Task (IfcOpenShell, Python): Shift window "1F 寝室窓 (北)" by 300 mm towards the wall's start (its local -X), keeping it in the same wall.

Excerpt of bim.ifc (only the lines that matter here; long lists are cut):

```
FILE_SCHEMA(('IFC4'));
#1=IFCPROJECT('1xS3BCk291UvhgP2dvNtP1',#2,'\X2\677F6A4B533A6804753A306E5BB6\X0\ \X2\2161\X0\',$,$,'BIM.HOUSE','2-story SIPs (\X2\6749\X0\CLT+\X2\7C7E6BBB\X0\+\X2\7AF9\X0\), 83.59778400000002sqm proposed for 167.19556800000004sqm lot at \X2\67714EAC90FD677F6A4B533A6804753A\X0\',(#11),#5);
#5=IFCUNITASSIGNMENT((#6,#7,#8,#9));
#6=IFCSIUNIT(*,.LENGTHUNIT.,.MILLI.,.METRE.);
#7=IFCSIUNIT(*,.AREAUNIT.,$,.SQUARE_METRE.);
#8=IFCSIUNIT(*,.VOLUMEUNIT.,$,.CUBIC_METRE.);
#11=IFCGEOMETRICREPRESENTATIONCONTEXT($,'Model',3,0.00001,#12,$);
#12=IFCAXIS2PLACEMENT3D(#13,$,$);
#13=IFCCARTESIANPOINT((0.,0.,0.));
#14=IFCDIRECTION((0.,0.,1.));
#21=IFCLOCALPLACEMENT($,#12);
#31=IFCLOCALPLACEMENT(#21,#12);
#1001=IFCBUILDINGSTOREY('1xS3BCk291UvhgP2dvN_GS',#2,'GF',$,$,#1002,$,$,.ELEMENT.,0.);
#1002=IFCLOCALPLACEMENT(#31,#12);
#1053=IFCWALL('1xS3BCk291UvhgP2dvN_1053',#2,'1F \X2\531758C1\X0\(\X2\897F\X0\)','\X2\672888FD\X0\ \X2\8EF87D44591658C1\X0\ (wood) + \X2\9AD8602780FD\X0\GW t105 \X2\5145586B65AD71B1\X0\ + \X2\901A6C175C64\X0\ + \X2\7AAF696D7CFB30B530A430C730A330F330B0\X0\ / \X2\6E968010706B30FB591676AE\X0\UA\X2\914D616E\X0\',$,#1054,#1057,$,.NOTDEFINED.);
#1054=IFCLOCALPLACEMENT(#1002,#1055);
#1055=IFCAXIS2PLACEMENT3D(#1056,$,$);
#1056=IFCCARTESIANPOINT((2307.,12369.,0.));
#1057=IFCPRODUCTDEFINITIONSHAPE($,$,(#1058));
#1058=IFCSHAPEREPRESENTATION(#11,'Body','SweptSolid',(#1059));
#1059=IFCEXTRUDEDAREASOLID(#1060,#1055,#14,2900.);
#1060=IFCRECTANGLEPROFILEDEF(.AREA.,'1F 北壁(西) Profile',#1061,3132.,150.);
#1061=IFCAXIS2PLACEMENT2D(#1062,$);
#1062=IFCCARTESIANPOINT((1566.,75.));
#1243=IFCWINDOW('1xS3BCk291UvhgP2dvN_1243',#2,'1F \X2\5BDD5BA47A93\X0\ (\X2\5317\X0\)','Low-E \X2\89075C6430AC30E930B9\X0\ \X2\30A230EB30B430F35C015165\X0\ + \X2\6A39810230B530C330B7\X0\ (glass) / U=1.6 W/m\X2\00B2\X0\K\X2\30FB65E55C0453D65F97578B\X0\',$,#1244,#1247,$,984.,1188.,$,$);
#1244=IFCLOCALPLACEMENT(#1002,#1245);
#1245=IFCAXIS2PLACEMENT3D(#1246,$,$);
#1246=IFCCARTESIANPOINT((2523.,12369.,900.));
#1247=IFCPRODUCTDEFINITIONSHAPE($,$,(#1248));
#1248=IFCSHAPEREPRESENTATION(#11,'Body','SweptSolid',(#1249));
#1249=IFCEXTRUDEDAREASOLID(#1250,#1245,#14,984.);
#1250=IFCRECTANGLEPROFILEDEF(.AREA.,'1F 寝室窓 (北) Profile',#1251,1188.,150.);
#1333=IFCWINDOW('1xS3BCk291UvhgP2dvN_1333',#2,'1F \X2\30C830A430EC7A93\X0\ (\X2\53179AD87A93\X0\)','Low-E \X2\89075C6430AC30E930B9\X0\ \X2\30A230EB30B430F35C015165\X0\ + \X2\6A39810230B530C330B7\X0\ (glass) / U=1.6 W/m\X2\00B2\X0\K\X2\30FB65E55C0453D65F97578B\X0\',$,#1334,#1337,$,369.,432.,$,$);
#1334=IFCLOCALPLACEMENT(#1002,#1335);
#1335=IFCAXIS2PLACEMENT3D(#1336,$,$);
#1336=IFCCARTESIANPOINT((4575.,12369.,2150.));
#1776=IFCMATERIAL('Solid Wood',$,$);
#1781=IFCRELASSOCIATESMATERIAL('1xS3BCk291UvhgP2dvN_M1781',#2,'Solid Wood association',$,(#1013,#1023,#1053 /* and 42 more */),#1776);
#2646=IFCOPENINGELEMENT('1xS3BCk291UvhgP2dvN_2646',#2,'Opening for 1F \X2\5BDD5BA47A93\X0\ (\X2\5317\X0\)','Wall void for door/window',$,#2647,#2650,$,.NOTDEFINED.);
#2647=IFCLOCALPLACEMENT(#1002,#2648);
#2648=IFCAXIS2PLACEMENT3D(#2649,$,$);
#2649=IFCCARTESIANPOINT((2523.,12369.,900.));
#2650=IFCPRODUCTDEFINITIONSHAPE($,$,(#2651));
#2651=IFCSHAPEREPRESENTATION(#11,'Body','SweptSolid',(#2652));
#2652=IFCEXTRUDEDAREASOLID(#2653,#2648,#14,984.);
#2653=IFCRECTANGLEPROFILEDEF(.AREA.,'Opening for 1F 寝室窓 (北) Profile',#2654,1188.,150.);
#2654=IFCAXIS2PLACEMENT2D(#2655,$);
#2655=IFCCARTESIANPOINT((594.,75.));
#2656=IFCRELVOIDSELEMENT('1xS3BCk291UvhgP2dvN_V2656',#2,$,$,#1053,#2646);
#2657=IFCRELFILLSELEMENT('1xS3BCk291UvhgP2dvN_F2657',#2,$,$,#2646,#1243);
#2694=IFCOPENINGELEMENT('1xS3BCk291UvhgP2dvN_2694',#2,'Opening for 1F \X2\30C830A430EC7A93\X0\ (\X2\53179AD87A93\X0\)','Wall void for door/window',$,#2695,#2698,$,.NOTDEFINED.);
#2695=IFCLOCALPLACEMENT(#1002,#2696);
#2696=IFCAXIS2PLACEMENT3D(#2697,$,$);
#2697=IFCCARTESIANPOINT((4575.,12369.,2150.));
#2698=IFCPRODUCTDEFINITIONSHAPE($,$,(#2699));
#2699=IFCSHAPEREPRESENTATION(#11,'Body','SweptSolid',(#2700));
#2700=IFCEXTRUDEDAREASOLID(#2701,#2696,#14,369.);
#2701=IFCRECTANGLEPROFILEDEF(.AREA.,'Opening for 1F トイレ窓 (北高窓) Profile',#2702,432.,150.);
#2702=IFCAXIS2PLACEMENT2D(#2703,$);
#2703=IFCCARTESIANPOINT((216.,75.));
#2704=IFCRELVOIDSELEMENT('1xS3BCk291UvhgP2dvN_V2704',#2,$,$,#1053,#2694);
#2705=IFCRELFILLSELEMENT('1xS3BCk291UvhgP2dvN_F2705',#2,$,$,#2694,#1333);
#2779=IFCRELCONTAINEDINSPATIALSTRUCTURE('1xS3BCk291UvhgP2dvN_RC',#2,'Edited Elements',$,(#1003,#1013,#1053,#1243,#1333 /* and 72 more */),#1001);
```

```python
import ifcopenshell
import ifcopenshell.api.geometry
import ifcopenshell.util.placement

model = ifcopenshell.open("bim.ifc")

window = model.by_guid("1xS3BCk291UvhgP2dvN_1243")
opening = window.FillsVoids[0].RelatingOpeningElement
wall = opening.VoidsElements[0].RelatingBuildingElement

wall_matrix = ifcopenshell.util.placement.get_local_placement(wall.ObjectPlacement)
shift = wall_matrix[:3, 0] * -300.0
before = ifcopenshell.util.placement.get_local_placement(window.ObjectPlacement)[:3, 3].copy()

# The window is not placed relative to its opening, so move both.
for product in (opening, window):
    matrix = ifcopenshell.util.placement.get_local_placement(product.ObjectPlacement)
    matrix[:3, 3] += shift
    ifcopenshell.api.geometry.edit_object_placement(model, product=product, matrix=matrix, is_si=False)

after = ifcopenshell.util.placement.get_local_placement(window.ObjectPlacement)[:3, 3]
print("window moved by", (after - before).round(3) + 0.0)

model.write("bim_updated.ifc")
```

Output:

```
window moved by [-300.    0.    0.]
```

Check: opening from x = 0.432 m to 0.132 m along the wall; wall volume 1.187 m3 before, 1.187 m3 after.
